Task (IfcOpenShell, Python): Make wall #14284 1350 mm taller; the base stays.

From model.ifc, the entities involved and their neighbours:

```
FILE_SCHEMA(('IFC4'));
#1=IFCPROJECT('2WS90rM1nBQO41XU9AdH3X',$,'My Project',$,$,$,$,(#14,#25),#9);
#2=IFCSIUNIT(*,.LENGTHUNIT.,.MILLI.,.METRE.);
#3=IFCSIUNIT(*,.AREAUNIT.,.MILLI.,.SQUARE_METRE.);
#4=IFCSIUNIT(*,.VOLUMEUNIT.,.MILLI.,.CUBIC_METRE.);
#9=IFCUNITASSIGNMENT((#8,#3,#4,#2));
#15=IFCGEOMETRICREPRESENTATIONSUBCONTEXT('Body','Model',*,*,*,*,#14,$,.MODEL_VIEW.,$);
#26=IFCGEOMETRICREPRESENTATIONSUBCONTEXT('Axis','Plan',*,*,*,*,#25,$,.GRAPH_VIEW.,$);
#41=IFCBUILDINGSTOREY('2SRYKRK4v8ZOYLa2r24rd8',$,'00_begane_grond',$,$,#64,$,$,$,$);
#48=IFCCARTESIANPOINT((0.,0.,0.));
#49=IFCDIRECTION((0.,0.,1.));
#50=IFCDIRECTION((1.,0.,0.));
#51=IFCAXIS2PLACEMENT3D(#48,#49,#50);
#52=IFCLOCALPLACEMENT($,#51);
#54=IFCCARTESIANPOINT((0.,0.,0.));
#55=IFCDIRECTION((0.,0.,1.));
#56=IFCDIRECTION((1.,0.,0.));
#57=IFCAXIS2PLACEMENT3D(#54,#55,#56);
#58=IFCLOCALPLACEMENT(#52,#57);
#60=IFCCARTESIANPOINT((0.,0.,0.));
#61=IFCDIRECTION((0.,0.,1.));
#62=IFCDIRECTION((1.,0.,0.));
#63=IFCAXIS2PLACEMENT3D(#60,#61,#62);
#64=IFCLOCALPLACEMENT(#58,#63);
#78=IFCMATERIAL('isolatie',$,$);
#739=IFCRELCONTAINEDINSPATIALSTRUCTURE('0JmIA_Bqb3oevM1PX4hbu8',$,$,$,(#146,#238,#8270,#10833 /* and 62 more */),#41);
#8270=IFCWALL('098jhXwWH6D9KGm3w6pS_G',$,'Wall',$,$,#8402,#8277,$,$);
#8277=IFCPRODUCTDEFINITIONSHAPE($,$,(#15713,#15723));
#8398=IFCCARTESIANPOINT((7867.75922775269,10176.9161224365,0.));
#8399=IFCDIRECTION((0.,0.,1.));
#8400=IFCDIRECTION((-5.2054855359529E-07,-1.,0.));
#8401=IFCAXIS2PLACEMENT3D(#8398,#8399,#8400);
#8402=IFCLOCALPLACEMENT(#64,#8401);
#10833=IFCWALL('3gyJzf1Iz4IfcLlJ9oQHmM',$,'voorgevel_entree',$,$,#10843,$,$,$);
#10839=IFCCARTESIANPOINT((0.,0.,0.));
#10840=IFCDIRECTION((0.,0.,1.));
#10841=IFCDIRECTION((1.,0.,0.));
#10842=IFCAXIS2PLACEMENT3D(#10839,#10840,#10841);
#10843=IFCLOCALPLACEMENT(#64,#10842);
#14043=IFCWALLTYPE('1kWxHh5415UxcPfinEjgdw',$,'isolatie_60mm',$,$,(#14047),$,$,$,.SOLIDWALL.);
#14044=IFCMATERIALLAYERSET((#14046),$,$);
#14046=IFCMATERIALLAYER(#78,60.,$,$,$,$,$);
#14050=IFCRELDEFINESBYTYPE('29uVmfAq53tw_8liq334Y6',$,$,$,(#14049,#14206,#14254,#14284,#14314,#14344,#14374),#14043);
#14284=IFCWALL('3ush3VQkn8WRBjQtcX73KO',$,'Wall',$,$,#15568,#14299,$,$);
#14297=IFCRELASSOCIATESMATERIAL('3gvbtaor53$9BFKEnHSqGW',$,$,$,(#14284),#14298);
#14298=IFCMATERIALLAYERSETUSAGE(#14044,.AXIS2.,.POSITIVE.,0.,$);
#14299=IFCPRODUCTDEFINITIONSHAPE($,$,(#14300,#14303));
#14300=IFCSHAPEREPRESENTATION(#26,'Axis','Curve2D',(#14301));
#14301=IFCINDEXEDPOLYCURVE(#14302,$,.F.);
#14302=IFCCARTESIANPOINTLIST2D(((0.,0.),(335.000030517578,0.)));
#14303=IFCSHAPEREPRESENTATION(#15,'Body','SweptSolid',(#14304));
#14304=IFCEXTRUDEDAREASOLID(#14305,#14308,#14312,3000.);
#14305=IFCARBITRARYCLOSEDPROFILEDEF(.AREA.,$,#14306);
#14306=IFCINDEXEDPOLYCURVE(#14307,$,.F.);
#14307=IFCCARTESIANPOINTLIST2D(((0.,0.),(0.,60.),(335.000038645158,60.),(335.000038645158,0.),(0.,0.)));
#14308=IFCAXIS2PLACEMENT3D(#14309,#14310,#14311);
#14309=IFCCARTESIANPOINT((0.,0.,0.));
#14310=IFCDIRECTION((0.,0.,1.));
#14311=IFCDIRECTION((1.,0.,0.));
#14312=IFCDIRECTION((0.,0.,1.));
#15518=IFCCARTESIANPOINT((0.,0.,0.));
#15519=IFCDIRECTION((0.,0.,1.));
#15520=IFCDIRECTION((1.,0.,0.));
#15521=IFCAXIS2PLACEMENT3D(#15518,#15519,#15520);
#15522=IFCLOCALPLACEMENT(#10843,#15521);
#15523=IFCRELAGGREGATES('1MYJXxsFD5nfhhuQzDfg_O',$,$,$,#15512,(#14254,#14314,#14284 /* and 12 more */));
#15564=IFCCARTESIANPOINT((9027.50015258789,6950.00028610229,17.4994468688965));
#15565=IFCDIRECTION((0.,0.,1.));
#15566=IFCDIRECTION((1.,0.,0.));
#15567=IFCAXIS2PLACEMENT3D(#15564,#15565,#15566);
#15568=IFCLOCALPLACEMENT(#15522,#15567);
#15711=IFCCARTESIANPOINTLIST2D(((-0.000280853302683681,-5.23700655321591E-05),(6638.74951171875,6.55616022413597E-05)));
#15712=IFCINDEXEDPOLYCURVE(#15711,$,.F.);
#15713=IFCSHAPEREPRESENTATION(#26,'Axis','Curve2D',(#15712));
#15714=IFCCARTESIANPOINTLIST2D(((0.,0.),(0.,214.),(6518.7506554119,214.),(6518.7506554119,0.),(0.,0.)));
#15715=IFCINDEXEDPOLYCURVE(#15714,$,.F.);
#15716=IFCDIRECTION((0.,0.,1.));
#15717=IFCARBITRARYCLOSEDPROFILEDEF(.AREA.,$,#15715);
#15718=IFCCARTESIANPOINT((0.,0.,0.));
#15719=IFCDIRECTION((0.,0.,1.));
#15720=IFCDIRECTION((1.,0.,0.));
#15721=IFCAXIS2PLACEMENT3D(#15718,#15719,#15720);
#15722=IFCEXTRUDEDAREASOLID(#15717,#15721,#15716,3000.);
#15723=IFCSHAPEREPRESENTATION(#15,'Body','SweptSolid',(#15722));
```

```python
import ifcopenshell
import ifcopenshell.geom
import ifcopenshell.util.representation
import ifcopenshell.util.shape
import ifcopenshell.util.unit

model = ifcopenshell.open("model.ifc")
unit_scale = ifcopenshell.util.unit.calculate_unit_scale(model)
settings = ifcopenshell.geom.settings()


def volume(element):
    """Net volume in cubic metres, openings subtracted."""
    shape = ifcopenshell.geom.create_shape(settings, element)
    return ifcopenshell.util.shape.get_volume(shape.geometry)


wall = model.by_guid("3ush3VQkn8WRBjQtcX73KO")
before = volume(wall)

body = ifcopenshell.util.representation.get_representation(wall, "Model", "Body")
solid = body.Items[0]
old_height = solid.Depth
solid.Depth += 1.35 / unit_scale
after = volume(wall)

print(f"height {old_height:g} -> {solid.Depth:g}, volume {before:.3f} -> {after:.3f} m3")

model.write("model_v2.ifc")
```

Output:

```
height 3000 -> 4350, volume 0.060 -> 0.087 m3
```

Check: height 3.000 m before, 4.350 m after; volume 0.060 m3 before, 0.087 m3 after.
